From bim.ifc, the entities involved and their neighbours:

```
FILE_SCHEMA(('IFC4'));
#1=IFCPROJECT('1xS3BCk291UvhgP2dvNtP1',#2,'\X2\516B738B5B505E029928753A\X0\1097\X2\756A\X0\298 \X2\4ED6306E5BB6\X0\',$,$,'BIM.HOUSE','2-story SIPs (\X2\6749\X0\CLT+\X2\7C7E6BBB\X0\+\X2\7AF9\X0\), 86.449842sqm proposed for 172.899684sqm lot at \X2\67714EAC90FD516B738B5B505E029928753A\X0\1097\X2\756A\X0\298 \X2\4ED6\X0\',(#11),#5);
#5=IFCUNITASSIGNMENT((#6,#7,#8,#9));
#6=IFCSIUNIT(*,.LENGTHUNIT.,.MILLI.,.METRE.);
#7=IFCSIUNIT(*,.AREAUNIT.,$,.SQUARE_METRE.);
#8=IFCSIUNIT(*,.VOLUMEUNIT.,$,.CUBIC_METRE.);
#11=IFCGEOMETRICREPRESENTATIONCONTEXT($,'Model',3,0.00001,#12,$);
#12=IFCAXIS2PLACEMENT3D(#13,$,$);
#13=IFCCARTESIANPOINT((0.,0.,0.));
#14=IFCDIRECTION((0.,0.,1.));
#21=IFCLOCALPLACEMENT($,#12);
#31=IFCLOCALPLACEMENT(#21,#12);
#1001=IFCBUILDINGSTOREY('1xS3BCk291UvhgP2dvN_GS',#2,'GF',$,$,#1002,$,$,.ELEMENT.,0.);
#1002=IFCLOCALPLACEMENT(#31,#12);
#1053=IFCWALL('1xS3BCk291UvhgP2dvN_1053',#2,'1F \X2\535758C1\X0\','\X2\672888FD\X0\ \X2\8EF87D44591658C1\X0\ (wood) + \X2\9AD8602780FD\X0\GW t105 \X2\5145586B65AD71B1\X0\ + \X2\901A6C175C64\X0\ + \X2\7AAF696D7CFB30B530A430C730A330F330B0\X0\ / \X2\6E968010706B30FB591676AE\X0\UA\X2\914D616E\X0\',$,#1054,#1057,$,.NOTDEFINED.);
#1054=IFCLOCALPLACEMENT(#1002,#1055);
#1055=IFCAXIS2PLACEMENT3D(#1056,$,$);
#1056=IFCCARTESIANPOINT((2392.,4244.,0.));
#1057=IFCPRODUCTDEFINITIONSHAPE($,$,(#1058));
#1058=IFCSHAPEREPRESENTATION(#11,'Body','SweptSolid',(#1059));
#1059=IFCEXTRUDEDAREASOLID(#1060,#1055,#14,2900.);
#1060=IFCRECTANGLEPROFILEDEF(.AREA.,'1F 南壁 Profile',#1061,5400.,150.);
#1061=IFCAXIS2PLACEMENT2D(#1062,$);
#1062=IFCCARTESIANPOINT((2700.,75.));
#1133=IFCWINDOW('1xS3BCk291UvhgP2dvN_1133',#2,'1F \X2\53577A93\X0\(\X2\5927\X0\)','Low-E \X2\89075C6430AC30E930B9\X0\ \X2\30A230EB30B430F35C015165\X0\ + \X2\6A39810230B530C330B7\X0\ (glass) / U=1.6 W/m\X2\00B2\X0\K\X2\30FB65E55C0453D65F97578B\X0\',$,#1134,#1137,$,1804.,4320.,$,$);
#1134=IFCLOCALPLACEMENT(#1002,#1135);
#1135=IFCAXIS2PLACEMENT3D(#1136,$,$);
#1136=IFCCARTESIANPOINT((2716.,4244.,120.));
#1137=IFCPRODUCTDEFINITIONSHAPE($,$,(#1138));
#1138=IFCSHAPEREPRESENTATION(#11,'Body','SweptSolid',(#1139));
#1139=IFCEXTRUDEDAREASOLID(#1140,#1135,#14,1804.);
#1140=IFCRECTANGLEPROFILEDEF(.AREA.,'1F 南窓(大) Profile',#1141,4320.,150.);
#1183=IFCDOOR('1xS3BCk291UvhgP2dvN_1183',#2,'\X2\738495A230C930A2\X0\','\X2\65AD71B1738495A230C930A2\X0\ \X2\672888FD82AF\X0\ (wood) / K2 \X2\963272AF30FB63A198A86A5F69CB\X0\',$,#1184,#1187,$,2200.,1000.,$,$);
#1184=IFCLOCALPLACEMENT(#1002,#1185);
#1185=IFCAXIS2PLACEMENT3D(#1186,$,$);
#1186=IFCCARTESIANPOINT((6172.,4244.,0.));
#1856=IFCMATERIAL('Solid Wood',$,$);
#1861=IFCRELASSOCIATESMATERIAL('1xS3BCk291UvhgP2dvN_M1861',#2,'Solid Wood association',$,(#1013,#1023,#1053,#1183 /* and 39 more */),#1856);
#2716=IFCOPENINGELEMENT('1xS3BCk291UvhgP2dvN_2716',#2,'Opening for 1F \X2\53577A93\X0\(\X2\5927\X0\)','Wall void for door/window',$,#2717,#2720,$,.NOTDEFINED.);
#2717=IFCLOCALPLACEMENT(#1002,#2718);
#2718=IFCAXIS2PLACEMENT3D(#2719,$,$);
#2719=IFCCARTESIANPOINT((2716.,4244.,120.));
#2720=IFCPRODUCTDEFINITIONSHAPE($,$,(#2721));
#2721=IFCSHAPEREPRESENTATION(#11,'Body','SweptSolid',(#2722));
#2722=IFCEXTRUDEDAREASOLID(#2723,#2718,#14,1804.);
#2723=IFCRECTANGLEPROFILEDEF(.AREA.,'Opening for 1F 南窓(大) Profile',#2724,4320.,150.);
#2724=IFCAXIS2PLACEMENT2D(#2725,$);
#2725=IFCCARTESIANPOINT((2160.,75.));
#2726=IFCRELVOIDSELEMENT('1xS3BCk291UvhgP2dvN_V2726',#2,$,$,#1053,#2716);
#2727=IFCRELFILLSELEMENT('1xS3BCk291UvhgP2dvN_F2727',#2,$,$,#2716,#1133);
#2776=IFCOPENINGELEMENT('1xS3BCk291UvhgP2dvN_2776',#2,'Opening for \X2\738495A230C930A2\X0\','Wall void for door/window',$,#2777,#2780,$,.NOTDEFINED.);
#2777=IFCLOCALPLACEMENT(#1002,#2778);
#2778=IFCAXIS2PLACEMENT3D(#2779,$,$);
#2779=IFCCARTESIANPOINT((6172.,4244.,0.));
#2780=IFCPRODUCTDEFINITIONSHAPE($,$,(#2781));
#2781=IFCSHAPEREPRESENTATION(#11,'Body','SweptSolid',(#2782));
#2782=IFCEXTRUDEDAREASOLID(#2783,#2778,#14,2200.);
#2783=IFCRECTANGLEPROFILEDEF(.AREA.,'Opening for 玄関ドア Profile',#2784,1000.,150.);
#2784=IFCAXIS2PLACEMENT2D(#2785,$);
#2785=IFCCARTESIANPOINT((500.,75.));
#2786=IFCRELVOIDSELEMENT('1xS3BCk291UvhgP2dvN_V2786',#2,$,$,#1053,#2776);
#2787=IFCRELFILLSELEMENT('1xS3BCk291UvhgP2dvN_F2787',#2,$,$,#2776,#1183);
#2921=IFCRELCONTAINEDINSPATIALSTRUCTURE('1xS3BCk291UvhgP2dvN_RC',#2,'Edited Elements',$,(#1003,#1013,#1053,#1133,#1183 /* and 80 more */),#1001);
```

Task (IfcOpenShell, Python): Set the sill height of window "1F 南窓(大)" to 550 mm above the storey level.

```python
import numpy as np
import ifcopenshell
import ifcopenshell.api.geometry
import ifcopenshell.geom
import ifcopenshell.util.element
import ifcopenshell.util.placement
import ifcopenshell.util.shape
import ifcopenshell.util.unit

model = ifcopenshell.open("bim.ifc")
unit_scale = ifcopenshell.util.unit.calculate_unit_scale(model)

window = model.by_guid("1xS3BCk291UvhgP2dvN_1133")
opening = window.FillsVoids[0].RelatingOpeningElement
storey = ifcopenshell.util.element.get_container(window, ifc_class="IfcBuildingStorey")
level = ifcopenshell.util.placement.get_local_placement(storey.ObjectPlacement)[2, 3]

# The opening's origin need not be at the sill, so measure its lowest point.
shape = ifcopenshell.geom.create_shape(ifcopenshell.geom.settings(), opening)
bottom = ifcopenshell.util.shape.get_shape_bottom_elevation(shape, shape.geometry) / unit_scale
dz = level + 550.0 - bottom

shift = np.array([0.0, 0.0, dz])
# The window is not placed relative to its opening, so move both.
for product in (opening, window):
    matrix = ifcopenshell.util.placement.get_local_placement(product.ObjectPlacement)
    matrix[:3, 3] += shift
    ifcopenshell.api.geometry.edit_object_placement(model, product=product, matrix=matrix, is_si=False)

print(f"moved by {dz * unit_scale:+.3f} m")

model.write("bim_rev.ifc")
```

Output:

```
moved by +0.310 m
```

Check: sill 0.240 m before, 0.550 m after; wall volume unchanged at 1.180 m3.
